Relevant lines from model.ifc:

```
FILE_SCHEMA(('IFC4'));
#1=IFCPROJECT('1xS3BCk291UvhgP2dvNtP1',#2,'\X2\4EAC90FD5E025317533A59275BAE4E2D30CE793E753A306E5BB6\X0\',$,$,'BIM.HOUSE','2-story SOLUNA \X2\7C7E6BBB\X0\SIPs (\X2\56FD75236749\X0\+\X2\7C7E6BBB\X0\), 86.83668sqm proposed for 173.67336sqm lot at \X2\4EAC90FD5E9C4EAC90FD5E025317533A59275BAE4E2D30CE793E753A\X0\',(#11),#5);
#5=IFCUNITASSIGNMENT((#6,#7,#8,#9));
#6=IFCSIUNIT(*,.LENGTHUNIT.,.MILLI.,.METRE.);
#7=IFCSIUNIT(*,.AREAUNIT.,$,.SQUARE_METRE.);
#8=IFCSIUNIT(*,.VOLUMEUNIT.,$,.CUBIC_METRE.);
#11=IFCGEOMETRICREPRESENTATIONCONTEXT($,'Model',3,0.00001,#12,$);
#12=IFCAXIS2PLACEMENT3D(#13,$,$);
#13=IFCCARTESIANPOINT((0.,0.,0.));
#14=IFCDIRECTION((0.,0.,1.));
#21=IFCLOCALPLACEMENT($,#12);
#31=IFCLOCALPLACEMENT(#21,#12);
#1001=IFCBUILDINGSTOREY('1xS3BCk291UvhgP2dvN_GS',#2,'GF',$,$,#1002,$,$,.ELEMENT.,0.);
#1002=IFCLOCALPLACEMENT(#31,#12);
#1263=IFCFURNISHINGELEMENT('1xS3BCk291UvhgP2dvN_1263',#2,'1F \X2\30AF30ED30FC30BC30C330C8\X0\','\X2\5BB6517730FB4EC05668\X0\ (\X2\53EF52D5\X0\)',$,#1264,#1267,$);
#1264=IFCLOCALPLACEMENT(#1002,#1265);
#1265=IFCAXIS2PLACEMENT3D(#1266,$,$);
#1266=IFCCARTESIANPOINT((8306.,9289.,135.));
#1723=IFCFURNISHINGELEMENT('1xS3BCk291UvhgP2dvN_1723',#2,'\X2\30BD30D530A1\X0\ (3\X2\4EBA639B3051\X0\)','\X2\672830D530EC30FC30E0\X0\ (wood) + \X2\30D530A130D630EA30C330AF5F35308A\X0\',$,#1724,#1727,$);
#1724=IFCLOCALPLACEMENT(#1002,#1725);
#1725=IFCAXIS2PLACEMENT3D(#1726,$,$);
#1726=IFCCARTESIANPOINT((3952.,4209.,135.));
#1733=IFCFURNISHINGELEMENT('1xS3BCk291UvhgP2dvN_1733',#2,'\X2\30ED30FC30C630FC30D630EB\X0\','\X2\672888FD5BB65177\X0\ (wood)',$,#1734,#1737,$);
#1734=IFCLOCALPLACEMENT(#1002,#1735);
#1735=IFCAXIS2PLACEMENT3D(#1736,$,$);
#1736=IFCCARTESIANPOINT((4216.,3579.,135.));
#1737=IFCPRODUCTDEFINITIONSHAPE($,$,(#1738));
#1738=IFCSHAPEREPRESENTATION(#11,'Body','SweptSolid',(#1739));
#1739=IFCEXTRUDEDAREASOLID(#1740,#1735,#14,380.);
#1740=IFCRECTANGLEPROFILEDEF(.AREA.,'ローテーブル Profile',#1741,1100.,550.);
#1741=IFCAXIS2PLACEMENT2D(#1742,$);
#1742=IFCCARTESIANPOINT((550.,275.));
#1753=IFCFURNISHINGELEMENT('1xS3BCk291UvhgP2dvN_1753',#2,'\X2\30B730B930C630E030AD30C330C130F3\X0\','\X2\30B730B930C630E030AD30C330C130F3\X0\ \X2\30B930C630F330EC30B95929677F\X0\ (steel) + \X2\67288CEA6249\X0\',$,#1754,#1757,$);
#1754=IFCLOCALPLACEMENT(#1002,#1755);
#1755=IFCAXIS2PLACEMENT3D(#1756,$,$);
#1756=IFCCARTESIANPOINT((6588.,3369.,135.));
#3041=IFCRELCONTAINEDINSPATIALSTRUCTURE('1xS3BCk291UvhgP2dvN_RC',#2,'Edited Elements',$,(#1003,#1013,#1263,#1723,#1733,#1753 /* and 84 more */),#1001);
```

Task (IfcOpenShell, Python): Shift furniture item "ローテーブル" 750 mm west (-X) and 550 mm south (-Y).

```python
import ifcopenshell
import ifcopenshell.api.geometry
import ifcopenshell.util.placement
import ifcopenshell.util.unit

model = ifcopenshell.open("model.ifc")
unit_scale = ifcopenshell.util.unit.calculate_unit_scale(model)

item = model.by_guid("1xS3BCk291UvhgP2dvN_1733")
matrix = ifcopenshell.util.placement.get_local_placement(item.ObjectPlacement)
matrix[0, 3] -= 0.75 / unit_scale
matrix[1, 3] -= 0.55 / unit_scale
ifcopenshell.api.geometry.edit_object_placement(model, product=item, matrix=matrix, is_si=False)

print(ifcopenshell.util.placement.get_local_placement(item.ObjectPlacement).round(3) + 0.0)

model.write("model-out.ifc")
```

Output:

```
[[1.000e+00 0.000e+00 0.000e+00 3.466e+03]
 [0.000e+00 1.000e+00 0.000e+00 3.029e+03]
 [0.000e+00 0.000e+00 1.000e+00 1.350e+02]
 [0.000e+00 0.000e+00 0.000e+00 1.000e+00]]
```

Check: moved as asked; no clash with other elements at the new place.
